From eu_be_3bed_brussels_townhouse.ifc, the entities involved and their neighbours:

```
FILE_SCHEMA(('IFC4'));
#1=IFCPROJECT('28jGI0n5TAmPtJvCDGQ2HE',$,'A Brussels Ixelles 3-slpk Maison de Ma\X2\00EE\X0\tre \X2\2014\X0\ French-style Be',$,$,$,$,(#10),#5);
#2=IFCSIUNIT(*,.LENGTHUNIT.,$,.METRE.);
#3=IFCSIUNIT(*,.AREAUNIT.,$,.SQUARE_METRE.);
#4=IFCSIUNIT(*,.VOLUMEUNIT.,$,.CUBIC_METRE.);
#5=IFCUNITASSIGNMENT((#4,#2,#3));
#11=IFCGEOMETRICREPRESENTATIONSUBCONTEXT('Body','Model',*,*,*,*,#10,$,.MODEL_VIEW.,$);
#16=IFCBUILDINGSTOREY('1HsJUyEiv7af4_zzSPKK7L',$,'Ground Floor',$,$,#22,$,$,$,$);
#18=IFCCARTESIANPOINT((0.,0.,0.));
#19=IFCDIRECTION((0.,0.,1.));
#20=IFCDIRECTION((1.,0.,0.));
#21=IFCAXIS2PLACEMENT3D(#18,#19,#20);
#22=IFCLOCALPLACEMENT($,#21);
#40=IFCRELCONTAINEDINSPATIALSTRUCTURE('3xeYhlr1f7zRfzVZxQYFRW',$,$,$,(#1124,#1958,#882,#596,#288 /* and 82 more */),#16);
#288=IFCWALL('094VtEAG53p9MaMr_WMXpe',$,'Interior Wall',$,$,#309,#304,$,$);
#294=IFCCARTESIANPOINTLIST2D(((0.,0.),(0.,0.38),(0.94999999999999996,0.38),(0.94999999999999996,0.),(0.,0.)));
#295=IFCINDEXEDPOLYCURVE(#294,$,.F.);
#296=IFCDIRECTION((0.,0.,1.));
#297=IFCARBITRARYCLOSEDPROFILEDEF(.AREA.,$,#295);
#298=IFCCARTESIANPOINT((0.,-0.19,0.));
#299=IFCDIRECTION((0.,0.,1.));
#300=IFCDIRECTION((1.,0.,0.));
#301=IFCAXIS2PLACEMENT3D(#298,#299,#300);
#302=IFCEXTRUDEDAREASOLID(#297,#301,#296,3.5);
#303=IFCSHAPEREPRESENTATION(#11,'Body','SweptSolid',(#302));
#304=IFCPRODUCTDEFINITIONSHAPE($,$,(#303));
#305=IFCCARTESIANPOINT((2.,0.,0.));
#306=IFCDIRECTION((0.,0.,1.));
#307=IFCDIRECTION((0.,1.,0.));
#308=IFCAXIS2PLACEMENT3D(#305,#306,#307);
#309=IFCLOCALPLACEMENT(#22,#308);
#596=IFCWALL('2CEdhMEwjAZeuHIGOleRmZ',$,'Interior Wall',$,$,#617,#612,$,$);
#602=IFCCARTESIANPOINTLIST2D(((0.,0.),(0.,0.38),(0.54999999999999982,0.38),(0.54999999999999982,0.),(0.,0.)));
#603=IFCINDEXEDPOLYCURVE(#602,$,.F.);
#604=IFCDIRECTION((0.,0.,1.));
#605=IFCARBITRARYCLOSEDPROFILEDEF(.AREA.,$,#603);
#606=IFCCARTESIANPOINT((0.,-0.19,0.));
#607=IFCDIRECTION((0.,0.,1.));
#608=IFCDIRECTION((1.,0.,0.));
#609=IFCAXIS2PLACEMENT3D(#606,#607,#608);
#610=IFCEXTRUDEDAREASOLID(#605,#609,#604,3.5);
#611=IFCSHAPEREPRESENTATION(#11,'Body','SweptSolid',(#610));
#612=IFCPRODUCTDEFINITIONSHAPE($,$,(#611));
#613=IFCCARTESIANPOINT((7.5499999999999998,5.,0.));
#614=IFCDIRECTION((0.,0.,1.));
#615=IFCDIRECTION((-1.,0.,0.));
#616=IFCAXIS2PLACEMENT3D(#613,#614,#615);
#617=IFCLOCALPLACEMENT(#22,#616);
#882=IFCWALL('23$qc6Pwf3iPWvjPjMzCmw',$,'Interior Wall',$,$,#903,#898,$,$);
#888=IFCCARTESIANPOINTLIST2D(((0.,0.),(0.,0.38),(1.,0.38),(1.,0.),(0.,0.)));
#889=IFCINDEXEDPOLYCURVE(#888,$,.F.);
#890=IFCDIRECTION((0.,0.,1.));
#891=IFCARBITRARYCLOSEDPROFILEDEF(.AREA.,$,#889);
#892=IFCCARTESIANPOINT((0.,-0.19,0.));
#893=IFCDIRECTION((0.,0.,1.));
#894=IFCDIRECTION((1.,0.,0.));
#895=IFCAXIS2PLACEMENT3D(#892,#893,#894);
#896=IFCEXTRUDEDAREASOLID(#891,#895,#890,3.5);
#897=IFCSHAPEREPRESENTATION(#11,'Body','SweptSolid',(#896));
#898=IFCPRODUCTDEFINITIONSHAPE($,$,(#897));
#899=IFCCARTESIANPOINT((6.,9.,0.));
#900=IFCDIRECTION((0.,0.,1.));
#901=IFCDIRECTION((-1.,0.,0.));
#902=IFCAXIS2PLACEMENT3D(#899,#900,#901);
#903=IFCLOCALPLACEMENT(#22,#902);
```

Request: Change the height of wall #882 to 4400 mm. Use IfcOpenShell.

```python
import ifcopenshell
import ifcopenshell.geom
import ifcopenshell.util.representation
import ifcopenshell.util.shape

model = ifcopenshell.open("eu_be_3bed_brussels_townhouse.ifc")
settings = ifcopenshell.geom.settings()


def volume(element):
    """Net volume in cubic metres, openings subtracted."""
    shape = ifcopenshell.geom.create_shape(settings, element)
    return ifcopenshell.util.shape.get_volume(shape.geometry)


wall = model.by_id(882)
before = volume(wall)

body = ifcopenshell.util.representation.get_representation(wall, "Model", "Body")
solid = body.Items[0]
old_height = solid.Depth
solid.Depth = 4.4
after = volume(wall)

print(f"height {old_height:g} -> {solid.Depth:g}, volume {before:.3f} -> {after:.3f} m3")

model.write("eu_be_3bed_brussels_townhouse_updated.ifc")
```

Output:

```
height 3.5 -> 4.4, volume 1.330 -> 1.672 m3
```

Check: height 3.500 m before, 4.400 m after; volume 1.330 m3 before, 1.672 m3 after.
